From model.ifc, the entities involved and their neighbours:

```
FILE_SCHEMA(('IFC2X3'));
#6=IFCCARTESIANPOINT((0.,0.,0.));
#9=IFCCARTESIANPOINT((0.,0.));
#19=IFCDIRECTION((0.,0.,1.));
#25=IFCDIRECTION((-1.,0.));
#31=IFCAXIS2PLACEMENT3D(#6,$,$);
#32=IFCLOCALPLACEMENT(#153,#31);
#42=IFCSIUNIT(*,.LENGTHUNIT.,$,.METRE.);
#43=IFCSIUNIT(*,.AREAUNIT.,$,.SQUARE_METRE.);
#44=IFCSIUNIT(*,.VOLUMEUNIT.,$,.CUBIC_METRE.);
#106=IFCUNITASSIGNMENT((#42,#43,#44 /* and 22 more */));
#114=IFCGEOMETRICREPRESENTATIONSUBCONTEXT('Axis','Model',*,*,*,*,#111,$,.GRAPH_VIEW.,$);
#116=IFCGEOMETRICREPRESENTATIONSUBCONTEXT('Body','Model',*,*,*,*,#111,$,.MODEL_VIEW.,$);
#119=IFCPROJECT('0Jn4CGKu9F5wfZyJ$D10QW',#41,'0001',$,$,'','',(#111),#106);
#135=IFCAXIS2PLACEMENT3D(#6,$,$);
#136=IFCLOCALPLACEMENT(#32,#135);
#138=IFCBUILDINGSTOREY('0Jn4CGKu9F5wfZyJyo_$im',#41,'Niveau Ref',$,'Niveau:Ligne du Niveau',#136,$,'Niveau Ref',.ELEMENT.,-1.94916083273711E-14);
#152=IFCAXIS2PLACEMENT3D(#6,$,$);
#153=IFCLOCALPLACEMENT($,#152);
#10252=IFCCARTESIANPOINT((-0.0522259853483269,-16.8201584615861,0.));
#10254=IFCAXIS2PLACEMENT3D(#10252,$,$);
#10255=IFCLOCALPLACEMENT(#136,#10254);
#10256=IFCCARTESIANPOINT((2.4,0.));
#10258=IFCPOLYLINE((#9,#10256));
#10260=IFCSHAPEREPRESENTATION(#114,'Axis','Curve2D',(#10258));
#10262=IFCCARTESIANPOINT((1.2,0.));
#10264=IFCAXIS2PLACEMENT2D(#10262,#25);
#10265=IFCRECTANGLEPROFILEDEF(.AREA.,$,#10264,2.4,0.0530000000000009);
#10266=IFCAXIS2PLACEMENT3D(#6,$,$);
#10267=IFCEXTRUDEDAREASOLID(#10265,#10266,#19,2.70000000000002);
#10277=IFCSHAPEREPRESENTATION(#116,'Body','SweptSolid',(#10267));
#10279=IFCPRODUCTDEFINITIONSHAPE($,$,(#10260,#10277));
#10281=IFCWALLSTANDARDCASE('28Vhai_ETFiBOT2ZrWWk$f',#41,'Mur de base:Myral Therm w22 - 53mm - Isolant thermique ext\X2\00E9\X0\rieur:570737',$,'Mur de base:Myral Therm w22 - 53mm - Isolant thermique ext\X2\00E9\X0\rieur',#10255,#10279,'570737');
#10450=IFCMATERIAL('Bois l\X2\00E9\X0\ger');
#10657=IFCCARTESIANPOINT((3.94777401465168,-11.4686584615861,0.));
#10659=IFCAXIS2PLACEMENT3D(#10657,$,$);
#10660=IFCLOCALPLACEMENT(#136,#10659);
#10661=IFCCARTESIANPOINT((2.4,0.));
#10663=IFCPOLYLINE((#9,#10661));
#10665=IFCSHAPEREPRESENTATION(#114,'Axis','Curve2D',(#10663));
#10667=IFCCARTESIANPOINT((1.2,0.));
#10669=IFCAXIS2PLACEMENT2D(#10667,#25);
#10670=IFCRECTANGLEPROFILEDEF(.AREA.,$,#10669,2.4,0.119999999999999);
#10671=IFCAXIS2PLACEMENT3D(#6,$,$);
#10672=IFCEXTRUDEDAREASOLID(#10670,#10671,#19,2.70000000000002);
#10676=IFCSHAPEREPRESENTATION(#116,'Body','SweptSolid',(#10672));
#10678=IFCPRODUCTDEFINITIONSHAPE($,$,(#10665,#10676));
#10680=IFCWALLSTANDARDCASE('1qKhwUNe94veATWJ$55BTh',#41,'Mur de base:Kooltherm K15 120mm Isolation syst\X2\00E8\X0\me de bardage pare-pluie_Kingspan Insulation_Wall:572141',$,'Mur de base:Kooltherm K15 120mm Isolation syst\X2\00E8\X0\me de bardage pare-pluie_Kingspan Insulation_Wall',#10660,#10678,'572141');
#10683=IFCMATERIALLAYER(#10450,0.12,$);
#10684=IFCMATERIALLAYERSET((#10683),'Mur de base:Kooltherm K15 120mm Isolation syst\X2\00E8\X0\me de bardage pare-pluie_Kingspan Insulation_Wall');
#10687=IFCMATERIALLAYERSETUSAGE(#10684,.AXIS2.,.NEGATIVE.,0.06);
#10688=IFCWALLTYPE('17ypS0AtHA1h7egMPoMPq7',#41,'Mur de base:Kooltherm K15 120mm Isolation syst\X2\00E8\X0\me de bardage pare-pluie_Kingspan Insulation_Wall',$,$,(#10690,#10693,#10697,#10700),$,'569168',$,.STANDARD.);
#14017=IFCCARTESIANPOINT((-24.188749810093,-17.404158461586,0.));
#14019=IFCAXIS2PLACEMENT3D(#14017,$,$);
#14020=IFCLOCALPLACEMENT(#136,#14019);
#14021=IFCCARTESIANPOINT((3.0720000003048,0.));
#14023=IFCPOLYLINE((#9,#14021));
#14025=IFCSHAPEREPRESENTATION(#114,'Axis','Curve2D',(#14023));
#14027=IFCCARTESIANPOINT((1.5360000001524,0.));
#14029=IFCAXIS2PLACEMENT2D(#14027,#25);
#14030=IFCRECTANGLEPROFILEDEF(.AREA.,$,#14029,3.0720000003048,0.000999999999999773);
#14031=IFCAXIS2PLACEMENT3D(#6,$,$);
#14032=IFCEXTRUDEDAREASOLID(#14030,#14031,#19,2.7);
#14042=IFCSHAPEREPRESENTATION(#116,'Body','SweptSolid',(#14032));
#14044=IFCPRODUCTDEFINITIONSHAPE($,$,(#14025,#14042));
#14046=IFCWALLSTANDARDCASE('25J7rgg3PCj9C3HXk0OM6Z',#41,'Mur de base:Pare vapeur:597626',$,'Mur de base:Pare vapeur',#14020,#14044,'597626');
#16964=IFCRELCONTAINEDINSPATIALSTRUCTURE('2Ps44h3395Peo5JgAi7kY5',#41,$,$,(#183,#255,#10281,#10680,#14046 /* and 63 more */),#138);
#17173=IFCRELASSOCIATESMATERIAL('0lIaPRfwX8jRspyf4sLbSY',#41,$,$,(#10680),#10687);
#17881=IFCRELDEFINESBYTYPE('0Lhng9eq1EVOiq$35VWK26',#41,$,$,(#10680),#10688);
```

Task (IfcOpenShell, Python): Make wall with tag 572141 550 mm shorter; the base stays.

```python
import ifcopenshell
import ifcopenshell.geom
import ifcopenshell.util.representation
import ifcopenshell.util.shape
import ifcopenshell.util.unit

model = ifcopenshell.open("model.ifc")
unit_scale = ifcopenshell.util.unit.calculate_unit_scale(model)
settings = ifcopenshell.geom.settings()


def volume(element):
    """Net volume in cubic metres, openings subtracted."""
    shape = ifcopenshell.geom.create_shape(settings, element)
    return ifcopenshell.util.shape.get_volume(shape.geometry)


wall = model.by_id(10680)
before = volume(wall)

body = ifcopenshell.util.representation.get_representation(wall, "Model", "Body")
solid = body.Items[0]
old_height = solid.Depth
solid.Depth -= 0.55 / unit_scale
after = volume(wall)

print(f"height {old_height:g} -> {solid.Depth:g}, volume {before:.3f} -> {after:.3f} m3")

model.write("model_v2.ifc")
```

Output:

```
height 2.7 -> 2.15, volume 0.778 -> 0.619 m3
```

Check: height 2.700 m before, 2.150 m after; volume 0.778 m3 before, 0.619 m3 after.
